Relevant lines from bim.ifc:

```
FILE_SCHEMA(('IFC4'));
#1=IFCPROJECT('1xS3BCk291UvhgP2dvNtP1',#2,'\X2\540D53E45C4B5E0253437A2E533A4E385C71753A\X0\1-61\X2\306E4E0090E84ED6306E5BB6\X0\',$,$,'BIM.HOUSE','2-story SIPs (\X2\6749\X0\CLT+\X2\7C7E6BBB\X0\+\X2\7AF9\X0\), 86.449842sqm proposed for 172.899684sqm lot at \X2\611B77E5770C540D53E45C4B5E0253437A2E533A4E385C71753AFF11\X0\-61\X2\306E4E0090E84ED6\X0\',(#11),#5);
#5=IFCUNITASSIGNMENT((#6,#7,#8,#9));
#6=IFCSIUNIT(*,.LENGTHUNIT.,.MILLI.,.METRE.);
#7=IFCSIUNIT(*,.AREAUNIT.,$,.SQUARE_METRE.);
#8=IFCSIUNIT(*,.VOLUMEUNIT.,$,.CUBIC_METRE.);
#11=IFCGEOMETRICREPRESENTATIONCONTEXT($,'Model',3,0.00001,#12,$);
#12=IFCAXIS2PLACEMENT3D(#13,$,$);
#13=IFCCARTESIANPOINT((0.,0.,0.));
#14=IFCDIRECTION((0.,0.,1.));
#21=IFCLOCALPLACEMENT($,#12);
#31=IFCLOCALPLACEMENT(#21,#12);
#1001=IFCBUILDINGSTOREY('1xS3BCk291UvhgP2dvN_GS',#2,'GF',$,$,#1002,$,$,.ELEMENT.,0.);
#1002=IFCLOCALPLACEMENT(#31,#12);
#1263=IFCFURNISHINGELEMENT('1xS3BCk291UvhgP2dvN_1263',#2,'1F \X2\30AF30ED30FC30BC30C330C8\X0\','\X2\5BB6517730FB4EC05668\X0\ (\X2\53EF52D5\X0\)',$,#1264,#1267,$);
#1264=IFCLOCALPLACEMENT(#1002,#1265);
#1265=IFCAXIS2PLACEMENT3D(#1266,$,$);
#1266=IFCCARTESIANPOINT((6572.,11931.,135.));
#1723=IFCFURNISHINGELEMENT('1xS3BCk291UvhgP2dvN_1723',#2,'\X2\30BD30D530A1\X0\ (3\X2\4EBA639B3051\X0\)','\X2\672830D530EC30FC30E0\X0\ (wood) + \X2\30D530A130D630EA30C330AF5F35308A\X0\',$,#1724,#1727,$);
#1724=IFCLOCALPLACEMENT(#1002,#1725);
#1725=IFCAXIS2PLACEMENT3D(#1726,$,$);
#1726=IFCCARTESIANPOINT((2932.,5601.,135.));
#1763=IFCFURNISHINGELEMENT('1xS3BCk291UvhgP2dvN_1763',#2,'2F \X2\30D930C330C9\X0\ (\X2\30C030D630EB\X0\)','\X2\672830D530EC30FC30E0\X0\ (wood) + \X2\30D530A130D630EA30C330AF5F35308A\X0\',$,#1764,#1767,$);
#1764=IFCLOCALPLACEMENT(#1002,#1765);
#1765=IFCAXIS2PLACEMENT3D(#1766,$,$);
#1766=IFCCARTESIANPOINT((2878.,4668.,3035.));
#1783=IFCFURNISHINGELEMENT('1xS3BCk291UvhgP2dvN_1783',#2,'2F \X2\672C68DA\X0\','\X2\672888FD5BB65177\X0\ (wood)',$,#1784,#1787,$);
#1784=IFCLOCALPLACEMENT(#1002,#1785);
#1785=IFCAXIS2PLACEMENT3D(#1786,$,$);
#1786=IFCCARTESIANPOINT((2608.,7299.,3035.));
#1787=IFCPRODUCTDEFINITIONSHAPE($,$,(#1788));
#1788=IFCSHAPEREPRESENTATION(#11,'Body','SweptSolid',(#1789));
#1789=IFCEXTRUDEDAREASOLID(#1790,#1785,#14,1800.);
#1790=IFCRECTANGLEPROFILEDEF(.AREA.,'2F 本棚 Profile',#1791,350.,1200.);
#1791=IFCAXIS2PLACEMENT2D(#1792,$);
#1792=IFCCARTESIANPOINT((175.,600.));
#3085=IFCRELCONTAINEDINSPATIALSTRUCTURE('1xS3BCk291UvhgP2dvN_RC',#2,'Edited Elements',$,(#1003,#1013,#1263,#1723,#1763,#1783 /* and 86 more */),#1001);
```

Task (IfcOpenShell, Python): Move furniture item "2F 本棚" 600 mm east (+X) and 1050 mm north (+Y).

```python
import ifcopenshell
import ifcopenshell.api.geometry
import ifcopenshell.util.placement
import ifcopenshell.util.unit

model = ifcopenshell.open("bim.ifc")
unit_scale = ifcopenshell.util.unit.calculate_unit_scale(model)

item = model.by_id(1783)
matrix = ifcopenshell.util.placement.get_local_placement(item.ObjectPlacement)
matrix[0, 3] += 0.6 / unit_scale
matrix[1, 3] += 1.05 / unit_scale
ifcopenshell.api.geometry.edit_object_placement(model, product=item, matrix=matrix, is_si=False)

print(ifcopenshell.util.placement.get_local_placement(item.ObjectPlacement).round(3) + 0.0)

model.write("bim-out.ifc")
```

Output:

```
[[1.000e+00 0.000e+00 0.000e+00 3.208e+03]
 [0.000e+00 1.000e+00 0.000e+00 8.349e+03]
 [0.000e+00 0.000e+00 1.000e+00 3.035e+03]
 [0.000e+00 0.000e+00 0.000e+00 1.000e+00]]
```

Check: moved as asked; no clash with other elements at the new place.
